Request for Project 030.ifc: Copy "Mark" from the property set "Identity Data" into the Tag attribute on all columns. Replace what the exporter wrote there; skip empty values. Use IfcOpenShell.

First a look at what the model holds.

```python
import ifcopenshell
import ifcopenshell.util.element

model = ifcopenshell.open("Project 030.ifc")
print(model.schema)
columns = model.by_type("IfcColumn")
print(len(columns), "columns")
for e in columns[:8]:
    source = ifcopenshell.util.element.get_pset(e, "Identity Data", "Mark")
    target = e.Tag
    print(e.id(), repr(source), repr(target), sep=" | ")
```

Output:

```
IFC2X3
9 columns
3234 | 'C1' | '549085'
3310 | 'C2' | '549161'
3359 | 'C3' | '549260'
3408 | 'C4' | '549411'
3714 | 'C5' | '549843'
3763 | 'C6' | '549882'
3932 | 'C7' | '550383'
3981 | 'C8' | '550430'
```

```python
import ifcopenshell
import ifcopenshell.util.element

model = ifcopenshell.open("Project 030.ifc")

count = 0
for e in model.by_type("IfcColumn"):
    value = ifcopenshell.util.element.get_pset(e, "Identity Data", "Mark")
    current = e.Tag
    if not value or not value.strip() or current == value:
        continue
    e.Tag = value
    count += 1

print(count, "columns updated")

model.write("Project 030_edited.ifc")
```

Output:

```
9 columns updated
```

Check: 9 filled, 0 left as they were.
